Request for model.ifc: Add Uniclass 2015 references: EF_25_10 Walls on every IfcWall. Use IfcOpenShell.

First a look at what the model holds.

```python
import ifcopenshell

model = ifcopenshell.open("model.ifc")
print(model.schema)
print("classifications:", [c.Name for c in model.by_type("IfcClassification")])
for ifc_class in ("IfcDoor", "IfcRoof", "IfcStair", "IfcWall", "IfcWindow"):
    print(ifc_class, len(model.by_type(ifc_class)))
```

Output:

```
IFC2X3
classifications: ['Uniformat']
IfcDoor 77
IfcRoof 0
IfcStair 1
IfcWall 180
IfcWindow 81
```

```python
import ifcopenshell
import ifcopenshell.api.classification

model = ifcopenshell.open("model.ifc")

# IFC2X3 requires Source and Edition and has no link from the project to the system.
system = model.create_entity("IfcClassification", Source="NBS", Edition="2015", Name="Uniclass 2015")

codes = {
    "IfcWall": ("EF_25_10", "Walls"),
}
for ifc_class, (code, name) in codes.items():
    products = model.by_type(ifc_class)
    ifcopenshell.api.classification.add_reference(
        model, products=products, classification=system, identification=code, name=name
    )
    print(code, len(products))

model.write("model_v2.ifc")
```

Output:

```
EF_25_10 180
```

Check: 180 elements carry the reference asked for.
